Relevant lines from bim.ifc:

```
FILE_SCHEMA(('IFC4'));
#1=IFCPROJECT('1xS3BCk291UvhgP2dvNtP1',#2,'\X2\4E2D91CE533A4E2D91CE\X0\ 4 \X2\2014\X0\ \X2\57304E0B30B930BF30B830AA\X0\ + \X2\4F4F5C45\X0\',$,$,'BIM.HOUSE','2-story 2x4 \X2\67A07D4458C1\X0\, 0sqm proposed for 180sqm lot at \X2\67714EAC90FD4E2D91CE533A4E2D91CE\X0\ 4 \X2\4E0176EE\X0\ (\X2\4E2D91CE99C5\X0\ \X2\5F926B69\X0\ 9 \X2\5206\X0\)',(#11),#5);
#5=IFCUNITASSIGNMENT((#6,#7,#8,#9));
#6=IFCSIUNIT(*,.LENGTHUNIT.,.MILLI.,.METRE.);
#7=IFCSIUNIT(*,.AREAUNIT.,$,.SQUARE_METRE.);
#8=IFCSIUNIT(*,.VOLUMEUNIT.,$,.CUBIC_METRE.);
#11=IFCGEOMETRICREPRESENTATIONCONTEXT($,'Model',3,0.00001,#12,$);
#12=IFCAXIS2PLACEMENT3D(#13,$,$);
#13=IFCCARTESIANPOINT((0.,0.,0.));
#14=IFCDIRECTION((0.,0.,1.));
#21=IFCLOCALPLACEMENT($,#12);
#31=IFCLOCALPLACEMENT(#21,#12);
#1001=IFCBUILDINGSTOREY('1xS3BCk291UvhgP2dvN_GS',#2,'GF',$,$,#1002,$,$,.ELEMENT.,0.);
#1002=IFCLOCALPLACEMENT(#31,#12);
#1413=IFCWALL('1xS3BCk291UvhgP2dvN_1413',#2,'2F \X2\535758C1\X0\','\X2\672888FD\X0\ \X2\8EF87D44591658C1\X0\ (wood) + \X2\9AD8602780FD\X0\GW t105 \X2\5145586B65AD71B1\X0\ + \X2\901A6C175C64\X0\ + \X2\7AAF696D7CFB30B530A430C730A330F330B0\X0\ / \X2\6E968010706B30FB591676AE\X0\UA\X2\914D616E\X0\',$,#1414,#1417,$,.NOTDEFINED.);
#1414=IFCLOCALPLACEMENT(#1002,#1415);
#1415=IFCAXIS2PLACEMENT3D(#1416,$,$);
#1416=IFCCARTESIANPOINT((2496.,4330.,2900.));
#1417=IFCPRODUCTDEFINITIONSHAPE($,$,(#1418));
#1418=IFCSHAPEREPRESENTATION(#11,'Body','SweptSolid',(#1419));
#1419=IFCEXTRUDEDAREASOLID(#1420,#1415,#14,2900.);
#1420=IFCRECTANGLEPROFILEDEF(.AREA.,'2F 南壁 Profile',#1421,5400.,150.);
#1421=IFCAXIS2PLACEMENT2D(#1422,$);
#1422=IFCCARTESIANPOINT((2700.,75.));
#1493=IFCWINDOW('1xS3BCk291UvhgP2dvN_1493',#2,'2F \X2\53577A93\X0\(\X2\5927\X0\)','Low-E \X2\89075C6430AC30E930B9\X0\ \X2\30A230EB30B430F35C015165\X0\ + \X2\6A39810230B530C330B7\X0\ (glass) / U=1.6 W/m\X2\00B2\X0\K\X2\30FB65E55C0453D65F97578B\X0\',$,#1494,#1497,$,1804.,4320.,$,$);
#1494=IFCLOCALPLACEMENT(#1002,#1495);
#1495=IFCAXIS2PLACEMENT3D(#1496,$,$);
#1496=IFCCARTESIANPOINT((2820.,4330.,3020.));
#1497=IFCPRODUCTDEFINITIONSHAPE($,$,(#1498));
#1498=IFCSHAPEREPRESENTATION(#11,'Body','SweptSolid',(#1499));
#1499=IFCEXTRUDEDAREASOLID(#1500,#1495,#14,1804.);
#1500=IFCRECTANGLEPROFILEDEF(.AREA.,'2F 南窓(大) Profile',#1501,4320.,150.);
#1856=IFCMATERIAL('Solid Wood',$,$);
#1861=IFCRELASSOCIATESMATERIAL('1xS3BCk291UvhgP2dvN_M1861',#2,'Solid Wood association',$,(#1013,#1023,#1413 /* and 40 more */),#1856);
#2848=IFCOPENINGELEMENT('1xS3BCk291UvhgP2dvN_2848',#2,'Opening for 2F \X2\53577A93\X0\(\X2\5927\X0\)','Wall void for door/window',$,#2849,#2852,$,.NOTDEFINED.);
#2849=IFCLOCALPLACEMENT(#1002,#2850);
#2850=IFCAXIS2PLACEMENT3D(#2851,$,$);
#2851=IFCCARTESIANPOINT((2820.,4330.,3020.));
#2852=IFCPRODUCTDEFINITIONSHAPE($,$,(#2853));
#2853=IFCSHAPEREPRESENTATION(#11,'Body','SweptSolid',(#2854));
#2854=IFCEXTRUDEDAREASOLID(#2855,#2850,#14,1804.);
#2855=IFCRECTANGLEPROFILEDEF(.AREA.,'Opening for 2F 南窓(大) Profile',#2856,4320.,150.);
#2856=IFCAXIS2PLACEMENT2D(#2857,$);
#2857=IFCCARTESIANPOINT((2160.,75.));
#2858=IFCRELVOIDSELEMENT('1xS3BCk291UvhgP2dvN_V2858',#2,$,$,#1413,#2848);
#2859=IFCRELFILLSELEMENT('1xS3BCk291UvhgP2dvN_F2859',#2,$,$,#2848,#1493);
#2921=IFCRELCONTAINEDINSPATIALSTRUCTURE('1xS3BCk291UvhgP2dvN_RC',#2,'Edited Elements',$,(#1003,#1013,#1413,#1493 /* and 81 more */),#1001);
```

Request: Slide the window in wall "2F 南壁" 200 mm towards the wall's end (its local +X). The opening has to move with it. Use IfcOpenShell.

```python
import ifcopenshell
import ifcopenshell.api.geometry
import ifcopenshell.util.placement
import ifcopenshell.util.unit

model = ifcopenshell.open("bim.ifc")
unit_scale = ifcopenshell.util.unit.calculate_unit_scale(model)

window = model.by_guid("1xS3BCk291UvhgP2dvN_1493")
opening = window.FillsVoids[0].RelatingOpeningElement
wall = opening.VoidsElements[0].RelatingBuildingElement

wall_matrix = ifcopenshell.util.placement.get_local_placement(wall.ObjectPlacement)
shift = wall_matrix[:3, 0] * 0.2 / unit_scale
before = ifcopenshell.util.placement.get_local_placement(window.ObjectPlacement)[:3, 3].copy()

# The window is not placed relative to its opening, so move both.
for product in (opening, window):
    matrix = ifcopenshell.util.placement.get_local_placement(product.ObjectPlacement)
    matrix[:3, 3] += shift
    ifcopenshell.api.geometry.edit_object_placement(model, product=product, matrix=matrix, is_si=False)

after = ifcopenshell.util.placement.get_local_placement(window.ObjectPlacement)[:3, 3]
print("window moved by", (after - before).round(3) + 0.0)

model.write("bim_v2.ifc")
```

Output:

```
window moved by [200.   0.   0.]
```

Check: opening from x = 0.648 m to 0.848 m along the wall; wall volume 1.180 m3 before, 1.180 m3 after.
